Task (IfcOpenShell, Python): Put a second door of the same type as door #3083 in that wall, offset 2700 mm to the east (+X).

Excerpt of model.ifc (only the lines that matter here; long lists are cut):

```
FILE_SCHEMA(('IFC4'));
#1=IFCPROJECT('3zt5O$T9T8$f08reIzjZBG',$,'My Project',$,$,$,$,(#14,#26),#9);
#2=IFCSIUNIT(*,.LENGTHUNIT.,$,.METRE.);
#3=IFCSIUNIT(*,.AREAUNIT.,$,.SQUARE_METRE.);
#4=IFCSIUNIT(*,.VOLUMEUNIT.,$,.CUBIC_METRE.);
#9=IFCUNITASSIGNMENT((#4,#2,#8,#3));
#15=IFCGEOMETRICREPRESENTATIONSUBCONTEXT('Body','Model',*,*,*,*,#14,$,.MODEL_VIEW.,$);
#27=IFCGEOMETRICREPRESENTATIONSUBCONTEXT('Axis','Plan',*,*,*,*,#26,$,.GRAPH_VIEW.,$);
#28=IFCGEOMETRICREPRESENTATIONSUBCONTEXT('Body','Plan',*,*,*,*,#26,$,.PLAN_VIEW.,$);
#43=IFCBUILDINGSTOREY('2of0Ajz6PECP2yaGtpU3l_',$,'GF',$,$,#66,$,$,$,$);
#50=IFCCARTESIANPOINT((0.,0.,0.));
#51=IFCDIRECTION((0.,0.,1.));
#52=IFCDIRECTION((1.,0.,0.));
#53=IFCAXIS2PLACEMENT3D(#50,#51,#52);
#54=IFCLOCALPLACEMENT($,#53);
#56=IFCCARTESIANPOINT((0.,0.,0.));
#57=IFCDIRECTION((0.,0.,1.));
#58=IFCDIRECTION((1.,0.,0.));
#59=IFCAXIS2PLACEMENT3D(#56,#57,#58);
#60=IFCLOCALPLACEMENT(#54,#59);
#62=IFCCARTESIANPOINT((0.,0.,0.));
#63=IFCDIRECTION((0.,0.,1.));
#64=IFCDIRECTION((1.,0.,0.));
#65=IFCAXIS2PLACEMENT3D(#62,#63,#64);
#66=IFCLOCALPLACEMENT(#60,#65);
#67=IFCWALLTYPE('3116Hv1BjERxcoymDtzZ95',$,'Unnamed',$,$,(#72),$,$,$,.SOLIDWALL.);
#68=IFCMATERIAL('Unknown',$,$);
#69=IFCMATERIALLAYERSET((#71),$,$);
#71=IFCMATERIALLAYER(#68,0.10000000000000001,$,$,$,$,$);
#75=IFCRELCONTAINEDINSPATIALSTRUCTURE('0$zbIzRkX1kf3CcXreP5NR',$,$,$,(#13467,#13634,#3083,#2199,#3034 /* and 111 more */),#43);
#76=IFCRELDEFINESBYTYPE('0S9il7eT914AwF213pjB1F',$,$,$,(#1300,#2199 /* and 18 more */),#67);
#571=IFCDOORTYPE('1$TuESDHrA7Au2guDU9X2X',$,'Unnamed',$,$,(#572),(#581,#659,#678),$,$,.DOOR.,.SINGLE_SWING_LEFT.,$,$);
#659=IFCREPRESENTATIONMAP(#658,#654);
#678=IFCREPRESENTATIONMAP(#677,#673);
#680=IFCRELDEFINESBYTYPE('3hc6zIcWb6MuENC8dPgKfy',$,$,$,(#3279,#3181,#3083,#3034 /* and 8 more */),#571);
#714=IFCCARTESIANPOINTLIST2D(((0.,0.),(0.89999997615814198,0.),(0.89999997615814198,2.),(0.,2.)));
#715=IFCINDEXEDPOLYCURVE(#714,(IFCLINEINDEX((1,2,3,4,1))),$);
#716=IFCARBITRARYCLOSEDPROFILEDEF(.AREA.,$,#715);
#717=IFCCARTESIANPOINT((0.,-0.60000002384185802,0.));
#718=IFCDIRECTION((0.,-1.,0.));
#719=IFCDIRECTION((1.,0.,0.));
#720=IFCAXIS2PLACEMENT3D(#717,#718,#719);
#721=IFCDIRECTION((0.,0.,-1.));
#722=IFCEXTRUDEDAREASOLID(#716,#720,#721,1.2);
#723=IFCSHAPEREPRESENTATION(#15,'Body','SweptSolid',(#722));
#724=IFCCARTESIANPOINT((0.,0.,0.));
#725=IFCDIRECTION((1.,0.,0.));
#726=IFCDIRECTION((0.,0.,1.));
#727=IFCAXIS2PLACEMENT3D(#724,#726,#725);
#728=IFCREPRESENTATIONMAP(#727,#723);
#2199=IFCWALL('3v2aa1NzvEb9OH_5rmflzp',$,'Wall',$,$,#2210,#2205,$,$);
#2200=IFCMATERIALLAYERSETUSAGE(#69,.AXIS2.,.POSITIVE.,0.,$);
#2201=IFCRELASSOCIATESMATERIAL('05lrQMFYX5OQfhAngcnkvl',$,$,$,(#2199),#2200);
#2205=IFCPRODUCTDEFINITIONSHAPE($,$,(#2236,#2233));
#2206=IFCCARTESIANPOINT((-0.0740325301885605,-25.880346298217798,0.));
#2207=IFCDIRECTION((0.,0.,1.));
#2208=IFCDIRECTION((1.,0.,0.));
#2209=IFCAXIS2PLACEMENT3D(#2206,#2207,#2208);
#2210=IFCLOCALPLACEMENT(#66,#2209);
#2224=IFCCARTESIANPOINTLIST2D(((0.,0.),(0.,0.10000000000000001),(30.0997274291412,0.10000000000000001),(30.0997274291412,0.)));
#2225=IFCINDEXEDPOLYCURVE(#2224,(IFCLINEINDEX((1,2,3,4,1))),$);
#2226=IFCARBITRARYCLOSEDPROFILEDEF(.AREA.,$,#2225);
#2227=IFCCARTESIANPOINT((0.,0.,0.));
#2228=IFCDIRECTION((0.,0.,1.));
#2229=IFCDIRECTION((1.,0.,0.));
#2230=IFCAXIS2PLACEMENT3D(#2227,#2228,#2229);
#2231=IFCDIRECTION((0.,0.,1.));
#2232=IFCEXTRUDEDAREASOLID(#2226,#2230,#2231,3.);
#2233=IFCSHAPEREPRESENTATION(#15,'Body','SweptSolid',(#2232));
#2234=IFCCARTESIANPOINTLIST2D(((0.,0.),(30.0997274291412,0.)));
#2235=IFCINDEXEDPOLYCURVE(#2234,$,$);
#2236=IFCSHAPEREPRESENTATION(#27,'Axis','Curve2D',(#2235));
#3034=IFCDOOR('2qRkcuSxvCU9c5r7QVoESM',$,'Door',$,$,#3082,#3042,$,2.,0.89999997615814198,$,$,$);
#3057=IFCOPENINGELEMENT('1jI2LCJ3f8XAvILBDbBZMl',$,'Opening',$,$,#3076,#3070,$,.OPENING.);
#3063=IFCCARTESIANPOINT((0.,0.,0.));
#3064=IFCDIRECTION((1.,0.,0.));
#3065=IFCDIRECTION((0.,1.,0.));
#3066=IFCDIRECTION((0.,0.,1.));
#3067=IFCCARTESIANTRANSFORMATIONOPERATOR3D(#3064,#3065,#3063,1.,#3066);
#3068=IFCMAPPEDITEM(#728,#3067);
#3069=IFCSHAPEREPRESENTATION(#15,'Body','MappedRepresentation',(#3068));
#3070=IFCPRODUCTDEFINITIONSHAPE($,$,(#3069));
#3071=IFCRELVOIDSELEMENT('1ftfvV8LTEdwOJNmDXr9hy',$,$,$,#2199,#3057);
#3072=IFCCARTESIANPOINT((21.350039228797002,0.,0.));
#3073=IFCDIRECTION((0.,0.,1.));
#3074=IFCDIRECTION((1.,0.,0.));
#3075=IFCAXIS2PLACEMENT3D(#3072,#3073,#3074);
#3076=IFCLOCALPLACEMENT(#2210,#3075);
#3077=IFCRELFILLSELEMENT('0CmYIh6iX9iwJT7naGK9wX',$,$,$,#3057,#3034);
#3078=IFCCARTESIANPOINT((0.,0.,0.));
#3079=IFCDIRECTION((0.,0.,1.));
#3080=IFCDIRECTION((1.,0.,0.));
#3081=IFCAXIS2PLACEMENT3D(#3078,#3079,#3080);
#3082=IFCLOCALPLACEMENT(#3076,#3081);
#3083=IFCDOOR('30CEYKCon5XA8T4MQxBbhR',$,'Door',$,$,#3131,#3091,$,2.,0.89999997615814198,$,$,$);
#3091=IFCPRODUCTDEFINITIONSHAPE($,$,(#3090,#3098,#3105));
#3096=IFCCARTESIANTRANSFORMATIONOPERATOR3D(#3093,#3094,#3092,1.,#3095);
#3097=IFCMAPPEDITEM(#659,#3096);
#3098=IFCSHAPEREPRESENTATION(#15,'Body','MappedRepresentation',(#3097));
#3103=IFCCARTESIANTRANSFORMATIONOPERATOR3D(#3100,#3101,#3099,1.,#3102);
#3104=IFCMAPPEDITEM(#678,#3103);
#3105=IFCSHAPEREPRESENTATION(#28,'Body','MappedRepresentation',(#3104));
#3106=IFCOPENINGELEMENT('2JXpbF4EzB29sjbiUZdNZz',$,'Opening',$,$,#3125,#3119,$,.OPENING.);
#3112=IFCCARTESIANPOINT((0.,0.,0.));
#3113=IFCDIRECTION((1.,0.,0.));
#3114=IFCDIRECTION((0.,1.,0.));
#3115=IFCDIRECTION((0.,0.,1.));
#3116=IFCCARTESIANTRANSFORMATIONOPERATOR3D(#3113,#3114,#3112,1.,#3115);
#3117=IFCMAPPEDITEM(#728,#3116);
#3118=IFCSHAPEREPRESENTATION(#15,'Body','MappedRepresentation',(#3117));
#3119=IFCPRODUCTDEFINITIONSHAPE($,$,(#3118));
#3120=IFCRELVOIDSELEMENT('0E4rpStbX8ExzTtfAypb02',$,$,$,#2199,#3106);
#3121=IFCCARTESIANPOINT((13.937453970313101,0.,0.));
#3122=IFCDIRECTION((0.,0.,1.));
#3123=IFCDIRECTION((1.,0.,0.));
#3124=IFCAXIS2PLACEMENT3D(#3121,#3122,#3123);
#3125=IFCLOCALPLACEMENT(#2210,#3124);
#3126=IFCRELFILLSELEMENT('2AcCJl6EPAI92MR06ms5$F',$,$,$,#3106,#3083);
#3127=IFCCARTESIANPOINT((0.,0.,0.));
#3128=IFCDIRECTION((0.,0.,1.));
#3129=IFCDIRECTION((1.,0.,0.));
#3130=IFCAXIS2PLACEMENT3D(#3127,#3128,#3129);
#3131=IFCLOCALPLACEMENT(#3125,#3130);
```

```python
import ifcopenshell
import ifcopenshell.api.feature
import ifcopenshell.api.geometry
import ifcopenshell.api.root
import ifcopenshell.geom
import ifcopenshell.util.element
import ifcopenshell.util.placement
import ifcopenshell.util.shape
import ifcopenshell.util.unit

model = ifcopenshell.open("model.ifc")
unit_scale = ifcopenshell.util.unit.calculate_unit_scale(model)
settings = ifcopenshell.geom.settings()


def volume(element):
    """Net volume in cubic metres, openings subtracted."""
    shape = ifcopenshell.geom.create_shape(settings, element)
    return ifcopenshell.util.shape.get_volume(shape.geometry)


door = model.by_guid("30CEYKCon5XA8T4MQxBbhR")
opening = door.FillsVoids[0].RelatingOpeningElement
wall = opening.VoidsElements[0].RelatingBuildingElement
before = volume(wall)
shift = ifcopenshell.util.placement.get_local_placement(wall.ObjectPlacement)[:3, 0] * 2.7 / unit_scale

# copy_class copies the void relationship, type, container and properties, but no geometry.
new_opening = ifcopenshell.api.root.copy_class(model, product=opening)
new_opening.Representation = ifcopenshell.util.element.copy_deep(
    model, opening.Representation, exclude=["IfcGeometricRepresentationContext", "IfcRepresentationMap"]
)
new_door = ifcopenshell.api.root.copy_class(model, product=door)
new_door.Representation = ifcopenshell.util.element.copy_deep(
    model, door.Representation, exclude=["IfcGeometricRepresentationContext", "IfcRepresentationMap"]
)
ifcopenshell.api.feature.add_filling(model, opening=new_opening, element=new_door)

for old, new in ((opening, new_opening), (door, new_door)):
    matrix = ifcopenshell.util.placement.get_local_placement(old.ObjectPlacement)
    matrix[:3, 3] += shift
    ifcopenshell.api.geometry.edit_object_placement(model, product=new, matrix=matrix, is_si=False)

after = volume(wall)

print(f"wall volume {before:.3f} -> {after:.3f} m3")

model.write("model_updated.ifc")
```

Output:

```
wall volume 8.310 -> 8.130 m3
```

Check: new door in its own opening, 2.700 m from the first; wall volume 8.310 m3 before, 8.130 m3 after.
